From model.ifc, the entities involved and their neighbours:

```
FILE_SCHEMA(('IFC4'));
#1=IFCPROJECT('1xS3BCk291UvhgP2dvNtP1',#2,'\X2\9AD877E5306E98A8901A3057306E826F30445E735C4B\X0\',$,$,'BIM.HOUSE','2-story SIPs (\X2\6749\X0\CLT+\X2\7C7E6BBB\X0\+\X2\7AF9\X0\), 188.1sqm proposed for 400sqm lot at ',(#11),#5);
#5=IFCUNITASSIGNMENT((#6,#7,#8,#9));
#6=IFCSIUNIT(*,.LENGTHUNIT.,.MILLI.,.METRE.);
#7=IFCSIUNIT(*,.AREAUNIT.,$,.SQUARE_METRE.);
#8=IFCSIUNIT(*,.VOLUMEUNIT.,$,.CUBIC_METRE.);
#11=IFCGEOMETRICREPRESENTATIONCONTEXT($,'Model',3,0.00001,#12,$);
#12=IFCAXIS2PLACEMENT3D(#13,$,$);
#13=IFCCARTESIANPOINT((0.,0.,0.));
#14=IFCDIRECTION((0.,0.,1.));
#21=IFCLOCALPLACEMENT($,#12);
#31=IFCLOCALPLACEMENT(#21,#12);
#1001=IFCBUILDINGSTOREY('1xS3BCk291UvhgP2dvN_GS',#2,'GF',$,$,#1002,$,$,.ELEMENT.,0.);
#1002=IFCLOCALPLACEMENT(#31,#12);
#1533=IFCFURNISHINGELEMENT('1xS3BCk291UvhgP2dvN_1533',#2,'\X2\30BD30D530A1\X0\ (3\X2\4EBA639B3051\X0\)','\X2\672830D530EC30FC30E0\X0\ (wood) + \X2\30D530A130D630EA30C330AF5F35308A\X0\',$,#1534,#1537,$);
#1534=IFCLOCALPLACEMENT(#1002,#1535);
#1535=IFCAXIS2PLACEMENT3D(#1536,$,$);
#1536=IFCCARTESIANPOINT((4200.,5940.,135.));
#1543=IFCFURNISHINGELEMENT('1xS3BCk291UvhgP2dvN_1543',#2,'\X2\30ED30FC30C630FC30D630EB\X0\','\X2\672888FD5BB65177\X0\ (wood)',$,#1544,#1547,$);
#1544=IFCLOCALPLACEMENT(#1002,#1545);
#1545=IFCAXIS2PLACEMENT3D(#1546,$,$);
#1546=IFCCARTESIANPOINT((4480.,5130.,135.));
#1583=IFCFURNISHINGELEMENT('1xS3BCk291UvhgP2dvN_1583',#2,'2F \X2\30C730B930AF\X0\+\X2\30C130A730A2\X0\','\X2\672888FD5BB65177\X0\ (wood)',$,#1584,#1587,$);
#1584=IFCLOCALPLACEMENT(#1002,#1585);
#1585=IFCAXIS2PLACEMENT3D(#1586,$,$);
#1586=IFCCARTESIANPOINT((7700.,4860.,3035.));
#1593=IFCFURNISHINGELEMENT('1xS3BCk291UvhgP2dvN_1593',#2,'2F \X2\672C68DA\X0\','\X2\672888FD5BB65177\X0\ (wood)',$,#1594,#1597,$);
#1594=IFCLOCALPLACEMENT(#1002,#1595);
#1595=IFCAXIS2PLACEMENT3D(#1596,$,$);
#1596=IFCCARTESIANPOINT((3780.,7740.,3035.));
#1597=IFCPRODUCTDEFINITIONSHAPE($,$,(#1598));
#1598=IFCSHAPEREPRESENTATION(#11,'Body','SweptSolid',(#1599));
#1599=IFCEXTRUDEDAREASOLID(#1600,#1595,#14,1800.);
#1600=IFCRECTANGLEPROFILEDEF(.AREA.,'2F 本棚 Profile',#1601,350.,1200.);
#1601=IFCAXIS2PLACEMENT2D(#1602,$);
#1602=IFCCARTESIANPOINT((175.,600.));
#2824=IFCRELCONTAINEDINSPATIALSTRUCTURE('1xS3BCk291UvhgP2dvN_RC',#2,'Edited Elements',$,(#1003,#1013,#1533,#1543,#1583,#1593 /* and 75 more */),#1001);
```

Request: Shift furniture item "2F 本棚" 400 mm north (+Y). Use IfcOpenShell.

```python
import ifcopenshell
import ifcopenshell.api.geometry
import ifcopenshell.util.placement

model = ifcopenshell.open("model.ifc")

item = model.by_guid("1xS3BCk291UvhgP2dvN_1593")
matrix = ifcopenshell.util.placement.get_local_placement(item.ObjectPlacement)
matrix[1, 3] += 400.0
ifcopenshell.api.geometry.edit_object_placement(model, product=item, matrix=matrix, is_si=False)

print(ifcopenshell.util.placement.get_local_placement(item.ObjectPlacement).round(3) + 0.0)

model.write("model_v2.ifc")
```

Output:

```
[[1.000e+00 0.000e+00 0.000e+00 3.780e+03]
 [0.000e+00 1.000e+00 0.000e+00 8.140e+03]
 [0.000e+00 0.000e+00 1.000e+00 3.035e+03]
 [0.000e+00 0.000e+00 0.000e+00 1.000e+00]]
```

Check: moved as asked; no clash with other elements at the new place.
